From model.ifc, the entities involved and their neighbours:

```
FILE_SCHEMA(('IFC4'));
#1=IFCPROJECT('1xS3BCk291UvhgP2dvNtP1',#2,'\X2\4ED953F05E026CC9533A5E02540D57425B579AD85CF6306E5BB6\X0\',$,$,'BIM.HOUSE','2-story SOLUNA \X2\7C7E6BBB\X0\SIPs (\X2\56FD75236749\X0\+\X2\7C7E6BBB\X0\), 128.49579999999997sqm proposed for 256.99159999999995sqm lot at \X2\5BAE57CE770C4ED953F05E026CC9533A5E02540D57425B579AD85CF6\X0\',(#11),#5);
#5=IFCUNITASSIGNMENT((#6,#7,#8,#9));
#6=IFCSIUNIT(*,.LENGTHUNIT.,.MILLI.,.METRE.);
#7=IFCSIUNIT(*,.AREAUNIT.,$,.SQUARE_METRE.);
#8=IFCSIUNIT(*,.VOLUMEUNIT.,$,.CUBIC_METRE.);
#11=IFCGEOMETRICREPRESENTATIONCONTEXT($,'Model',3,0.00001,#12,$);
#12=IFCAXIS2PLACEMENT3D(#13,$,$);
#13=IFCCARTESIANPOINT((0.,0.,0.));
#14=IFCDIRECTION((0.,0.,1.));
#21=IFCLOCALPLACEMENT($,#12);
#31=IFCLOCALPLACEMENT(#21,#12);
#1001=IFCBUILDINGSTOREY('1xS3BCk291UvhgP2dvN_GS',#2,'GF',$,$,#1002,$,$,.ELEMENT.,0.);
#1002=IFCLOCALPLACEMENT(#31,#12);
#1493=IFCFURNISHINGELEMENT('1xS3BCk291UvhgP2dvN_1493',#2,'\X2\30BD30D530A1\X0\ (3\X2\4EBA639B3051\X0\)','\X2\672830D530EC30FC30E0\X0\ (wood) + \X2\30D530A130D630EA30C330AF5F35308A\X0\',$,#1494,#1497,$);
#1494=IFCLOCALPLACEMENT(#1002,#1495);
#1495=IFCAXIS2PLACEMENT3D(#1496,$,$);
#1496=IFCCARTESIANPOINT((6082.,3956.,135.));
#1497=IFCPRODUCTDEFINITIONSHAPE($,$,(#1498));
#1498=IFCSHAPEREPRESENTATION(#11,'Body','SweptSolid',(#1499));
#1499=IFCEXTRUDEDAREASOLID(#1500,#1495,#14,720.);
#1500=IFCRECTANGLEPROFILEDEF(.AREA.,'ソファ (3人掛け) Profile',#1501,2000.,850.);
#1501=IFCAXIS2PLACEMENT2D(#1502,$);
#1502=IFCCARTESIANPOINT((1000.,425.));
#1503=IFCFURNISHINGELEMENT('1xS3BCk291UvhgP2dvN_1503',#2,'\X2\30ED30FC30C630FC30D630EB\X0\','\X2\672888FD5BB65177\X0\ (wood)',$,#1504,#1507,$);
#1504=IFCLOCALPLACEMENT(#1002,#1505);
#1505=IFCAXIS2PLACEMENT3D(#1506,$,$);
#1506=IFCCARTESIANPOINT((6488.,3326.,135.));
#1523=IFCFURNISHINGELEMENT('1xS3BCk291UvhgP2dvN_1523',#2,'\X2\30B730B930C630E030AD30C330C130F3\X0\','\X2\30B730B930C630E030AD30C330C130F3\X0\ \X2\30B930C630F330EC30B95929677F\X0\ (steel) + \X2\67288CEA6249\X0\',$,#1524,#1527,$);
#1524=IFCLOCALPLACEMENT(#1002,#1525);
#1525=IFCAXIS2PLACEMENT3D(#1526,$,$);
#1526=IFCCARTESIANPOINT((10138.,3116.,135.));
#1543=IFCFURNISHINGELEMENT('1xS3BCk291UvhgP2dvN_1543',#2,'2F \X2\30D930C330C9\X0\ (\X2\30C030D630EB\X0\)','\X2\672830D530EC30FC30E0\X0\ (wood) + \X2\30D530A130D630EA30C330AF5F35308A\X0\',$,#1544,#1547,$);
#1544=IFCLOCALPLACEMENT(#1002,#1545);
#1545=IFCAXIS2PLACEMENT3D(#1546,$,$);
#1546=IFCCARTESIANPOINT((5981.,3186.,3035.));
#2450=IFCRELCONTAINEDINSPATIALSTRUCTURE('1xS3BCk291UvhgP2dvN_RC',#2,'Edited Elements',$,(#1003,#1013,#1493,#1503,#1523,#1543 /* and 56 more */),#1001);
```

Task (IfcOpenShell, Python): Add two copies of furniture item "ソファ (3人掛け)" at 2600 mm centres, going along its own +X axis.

```python
import ifcopenshell
import ifcopenshell.api.geometry
import ifcopenshell.api.root
import ifcopenshell.util.element
import ifcopenshell.util.placement
import ifcopenshell.util.unit

model = ifcopenshell.open("model.ifc")
unit_scale = ifcopenshell.util.unit.calculate_unit_scale(model)


def reuse_history(source, copy):
    """copy_class also copies each property set's owner history, people and application; keep the originals."""
    for rel in copy.IsDefinedBy:
        if rel.is_a("IfcRelDefinesByProperties") and (history := rel.RelatingPropertyDefinition.OwnerHistory):
            rel.RelatingPropertyDefinition.OwnerHistory = source.OwnerHistory
            ifcopenshell.util.element.remove_deep2(model, history)


source = model.by_guid("1xS3BCk291UvhgP2dvN_1493")
base = ifcopenshell.util.placement.get_local_placement(source.ObjectPlacement)
step = base[:3, 0] * 2.6 / unit_scale

for i in range(1, 3):
    copy = ifcopenshell.api.root.copy_class(model, product=source)
    copy.Representation = ifcopenshell.util.element.copy_deep(
        model, source.Representation, exclude=["IfcGeometricRepresentationContext", "IfcRepresentationMap"]
    )
    reuse_history(source, copy)
    matrix = base.copy()
    matrix[:3, 3] += i * step
    print("added at", matrix[:3, 3].round(3) + 0.0)
    ifcopenshell.api.geometry.edit_object_placement(model, product=copy, matrix=matrix, is_si=False)

model.write("model_updated.ifc")
```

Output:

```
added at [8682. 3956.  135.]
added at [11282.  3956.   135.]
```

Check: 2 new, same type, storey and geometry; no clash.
